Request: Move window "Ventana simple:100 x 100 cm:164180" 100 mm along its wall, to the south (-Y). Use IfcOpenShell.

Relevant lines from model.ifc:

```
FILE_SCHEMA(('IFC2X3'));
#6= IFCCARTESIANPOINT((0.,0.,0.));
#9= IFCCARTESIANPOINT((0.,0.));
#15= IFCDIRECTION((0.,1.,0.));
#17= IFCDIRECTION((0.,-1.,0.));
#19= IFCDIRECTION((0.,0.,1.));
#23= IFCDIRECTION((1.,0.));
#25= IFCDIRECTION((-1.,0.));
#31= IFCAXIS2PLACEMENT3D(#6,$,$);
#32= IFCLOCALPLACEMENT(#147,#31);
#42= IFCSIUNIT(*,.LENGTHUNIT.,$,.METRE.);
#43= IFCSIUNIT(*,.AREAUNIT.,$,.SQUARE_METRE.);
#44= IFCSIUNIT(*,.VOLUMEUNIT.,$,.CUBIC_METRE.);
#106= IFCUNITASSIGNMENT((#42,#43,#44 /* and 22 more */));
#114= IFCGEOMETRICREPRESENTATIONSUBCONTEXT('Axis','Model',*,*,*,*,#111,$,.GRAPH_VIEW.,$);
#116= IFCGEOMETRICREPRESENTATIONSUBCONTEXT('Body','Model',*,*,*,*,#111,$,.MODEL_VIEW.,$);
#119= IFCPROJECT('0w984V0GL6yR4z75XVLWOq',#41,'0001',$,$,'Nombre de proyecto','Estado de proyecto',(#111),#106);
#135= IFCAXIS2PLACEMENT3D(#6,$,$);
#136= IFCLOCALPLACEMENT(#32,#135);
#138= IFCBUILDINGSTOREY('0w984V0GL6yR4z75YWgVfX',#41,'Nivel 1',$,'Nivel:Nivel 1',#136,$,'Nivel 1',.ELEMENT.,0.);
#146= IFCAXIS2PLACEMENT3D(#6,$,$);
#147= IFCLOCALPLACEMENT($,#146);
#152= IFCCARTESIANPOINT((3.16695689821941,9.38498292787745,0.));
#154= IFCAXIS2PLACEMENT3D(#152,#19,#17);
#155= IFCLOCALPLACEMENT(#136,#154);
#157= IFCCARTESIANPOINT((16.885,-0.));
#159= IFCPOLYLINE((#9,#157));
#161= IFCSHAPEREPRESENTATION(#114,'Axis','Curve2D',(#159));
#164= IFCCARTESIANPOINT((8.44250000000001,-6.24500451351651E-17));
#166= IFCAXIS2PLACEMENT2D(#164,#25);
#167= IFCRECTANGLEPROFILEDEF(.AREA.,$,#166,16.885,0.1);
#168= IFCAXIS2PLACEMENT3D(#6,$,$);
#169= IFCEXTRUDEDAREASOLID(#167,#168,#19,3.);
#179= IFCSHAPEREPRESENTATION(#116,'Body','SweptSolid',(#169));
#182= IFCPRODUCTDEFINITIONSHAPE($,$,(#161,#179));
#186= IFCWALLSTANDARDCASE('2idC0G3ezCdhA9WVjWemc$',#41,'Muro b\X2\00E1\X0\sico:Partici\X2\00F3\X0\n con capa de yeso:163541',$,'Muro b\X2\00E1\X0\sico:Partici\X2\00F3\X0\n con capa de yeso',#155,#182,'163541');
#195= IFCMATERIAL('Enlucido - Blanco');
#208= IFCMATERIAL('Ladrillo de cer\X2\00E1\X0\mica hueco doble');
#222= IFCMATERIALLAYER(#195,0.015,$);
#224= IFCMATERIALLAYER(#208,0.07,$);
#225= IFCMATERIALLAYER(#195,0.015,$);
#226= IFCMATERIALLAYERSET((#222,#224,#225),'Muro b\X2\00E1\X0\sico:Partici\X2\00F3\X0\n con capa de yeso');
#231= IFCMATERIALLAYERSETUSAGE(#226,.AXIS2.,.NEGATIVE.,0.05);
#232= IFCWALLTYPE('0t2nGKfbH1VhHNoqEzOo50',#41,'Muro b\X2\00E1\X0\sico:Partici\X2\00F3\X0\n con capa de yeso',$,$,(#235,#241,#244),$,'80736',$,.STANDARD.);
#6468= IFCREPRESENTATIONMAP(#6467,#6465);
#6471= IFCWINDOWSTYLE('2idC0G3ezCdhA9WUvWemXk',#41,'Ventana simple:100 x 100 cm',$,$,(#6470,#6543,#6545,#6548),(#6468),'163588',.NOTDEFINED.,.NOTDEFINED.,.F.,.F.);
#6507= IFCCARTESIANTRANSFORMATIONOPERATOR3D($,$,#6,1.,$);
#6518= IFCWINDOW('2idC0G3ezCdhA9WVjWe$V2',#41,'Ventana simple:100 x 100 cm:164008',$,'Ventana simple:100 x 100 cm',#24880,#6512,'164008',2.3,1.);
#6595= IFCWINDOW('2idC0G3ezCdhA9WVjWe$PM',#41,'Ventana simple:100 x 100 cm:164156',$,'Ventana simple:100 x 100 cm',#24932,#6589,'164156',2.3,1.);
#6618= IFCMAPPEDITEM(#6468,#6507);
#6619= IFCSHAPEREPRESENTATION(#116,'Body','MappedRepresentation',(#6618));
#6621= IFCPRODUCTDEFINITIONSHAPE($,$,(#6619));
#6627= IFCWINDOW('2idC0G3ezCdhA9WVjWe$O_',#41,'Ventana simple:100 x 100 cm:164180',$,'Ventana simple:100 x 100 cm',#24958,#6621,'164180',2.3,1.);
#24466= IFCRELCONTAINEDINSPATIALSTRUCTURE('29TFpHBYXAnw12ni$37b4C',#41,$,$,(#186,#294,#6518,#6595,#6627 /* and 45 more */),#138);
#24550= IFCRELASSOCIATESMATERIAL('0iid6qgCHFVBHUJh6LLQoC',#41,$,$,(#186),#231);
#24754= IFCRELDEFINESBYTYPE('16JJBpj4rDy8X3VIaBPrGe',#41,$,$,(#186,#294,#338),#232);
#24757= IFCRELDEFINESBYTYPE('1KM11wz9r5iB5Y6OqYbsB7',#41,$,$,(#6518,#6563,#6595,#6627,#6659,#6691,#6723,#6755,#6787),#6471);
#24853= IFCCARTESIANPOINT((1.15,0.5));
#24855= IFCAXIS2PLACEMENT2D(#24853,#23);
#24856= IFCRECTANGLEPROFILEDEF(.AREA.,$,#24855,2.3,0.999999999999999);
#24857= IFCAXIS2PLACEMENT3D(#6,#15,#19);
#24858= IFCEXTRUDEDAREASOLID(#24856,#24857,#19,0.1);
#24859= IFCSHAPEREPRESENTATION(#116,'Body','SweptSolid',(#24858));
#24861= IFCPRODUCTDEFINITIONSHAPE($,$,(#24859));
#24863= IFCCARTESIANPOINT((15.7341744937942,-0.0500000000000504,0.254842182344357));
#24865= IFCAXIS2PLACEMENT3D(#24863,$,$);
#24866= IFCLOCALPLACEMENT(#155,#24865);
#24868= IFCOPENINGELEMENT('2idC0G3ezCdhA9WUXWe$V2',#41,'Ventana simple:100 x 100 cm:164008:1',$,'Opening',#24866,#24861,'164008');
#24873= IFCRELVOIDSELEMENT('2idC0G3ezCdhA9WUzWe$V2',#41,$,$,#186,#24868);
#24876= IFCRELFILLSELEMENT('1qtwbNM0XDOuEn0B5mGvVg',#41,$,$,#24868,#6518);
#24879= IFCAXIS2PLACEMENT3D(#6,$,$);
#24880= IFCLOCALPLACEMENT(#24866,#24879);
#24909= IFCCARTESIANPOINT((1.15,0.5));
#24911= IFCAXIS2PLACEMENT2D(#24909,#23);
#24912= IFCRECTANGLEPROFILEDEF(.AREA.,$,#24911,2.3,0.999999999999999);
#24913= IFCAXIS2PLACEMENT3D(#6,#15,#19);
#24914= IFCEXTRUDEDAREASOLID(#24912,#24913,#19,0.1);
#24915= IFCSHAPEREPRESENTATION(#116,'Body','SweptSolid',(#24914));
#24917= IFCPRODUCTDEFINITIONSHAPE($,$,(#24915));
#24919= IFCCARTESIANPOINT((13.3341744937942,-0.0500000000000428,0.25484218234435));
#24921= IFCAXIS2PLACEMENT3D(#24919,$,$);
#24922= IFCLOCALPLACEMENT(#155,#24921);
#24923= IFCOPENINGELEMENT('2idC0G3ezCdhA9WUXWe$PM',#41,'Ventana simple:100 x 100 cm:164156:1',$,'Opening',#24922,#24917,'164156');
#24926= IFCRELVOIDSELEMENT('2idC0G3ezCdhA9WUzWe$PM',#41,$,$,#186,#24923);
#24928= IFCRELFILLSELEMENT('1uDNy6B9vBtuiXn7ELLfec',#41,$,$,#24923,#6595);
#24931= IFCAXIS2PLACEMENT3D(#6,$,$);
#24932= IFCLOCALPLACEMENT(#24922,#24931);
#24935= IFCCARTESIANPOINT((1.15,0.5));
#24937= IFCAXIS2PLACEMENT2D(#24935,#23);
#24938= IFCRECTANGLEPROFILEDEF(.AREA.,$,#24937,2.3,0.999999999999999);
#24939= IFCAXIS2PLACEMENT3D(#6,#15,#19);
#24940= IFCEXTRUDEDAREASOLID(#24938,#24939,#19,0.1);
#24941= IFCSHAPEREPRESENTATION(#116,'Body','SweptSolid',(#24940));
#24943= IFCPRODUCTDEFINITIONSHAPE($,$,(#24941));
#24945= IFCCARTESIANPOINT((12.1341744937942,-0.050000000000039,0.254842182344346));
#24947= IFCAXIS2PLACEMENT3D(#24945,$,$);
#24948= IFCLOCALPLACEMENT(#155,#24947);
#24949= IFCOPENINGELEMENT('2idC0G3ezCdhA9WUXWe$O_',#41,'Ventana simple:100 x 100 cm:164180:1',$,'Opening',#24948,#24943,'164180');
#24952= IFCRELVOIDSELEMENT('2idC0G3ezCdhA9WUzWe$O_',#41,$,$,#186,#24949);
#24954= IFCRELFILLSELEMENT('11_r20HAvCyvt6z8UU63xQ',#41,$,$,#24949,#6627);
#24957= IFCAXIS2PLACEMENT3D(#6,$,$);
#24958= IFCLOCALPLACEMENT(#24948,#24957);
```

```python
import ifcopenshell
import ifcopenshell.api.geometry
import ifcopenshell.util.placement
import ifcopenshell.util.unit

model = ifcopenshell.open("model.ifc")
unit_scale = ifcopenshell.util.unit.calculate_unit_scale(model)

window = model.by_id(6627)
opening = window.FillsVoids[0].RelatingOpeningElement
wall = opening.VoidsElements[0].RelatingBuildingElement

wall_matrix = ifcopenshell.util.placement.get_local_placement(wall.ObjectPlacement)
shift = wall_matrix[:3, 0] * 0.1 / unit_scale
before = ifcopenshell.util.placement.get_local_placement(window.ObjectPlacement)[:3, 3].copy()

# The window is placed relative to its opening, so it follows when the opening moves.
matrix = ifcopenshell.util.placement.get_local_placement(opening.ObjectPlacement)
matrix[:3, 3] += shift
ifcopenshell.api.geometry.edit_object_placement(
    model, product=opening, matrix=matrix, is_si=False, should_transform_children=True
)

after = ifcopenshell.util.placement.get_local_placement(window.ObjectPlacement)[:3, 3]
print("window moved by", (after - before).round(3) + 0.0)

model.write("model_updated.ifc")
```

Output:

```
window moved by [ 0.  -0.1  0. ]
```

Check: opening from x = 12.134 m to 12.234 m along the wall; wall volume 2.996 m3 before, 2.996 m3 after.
